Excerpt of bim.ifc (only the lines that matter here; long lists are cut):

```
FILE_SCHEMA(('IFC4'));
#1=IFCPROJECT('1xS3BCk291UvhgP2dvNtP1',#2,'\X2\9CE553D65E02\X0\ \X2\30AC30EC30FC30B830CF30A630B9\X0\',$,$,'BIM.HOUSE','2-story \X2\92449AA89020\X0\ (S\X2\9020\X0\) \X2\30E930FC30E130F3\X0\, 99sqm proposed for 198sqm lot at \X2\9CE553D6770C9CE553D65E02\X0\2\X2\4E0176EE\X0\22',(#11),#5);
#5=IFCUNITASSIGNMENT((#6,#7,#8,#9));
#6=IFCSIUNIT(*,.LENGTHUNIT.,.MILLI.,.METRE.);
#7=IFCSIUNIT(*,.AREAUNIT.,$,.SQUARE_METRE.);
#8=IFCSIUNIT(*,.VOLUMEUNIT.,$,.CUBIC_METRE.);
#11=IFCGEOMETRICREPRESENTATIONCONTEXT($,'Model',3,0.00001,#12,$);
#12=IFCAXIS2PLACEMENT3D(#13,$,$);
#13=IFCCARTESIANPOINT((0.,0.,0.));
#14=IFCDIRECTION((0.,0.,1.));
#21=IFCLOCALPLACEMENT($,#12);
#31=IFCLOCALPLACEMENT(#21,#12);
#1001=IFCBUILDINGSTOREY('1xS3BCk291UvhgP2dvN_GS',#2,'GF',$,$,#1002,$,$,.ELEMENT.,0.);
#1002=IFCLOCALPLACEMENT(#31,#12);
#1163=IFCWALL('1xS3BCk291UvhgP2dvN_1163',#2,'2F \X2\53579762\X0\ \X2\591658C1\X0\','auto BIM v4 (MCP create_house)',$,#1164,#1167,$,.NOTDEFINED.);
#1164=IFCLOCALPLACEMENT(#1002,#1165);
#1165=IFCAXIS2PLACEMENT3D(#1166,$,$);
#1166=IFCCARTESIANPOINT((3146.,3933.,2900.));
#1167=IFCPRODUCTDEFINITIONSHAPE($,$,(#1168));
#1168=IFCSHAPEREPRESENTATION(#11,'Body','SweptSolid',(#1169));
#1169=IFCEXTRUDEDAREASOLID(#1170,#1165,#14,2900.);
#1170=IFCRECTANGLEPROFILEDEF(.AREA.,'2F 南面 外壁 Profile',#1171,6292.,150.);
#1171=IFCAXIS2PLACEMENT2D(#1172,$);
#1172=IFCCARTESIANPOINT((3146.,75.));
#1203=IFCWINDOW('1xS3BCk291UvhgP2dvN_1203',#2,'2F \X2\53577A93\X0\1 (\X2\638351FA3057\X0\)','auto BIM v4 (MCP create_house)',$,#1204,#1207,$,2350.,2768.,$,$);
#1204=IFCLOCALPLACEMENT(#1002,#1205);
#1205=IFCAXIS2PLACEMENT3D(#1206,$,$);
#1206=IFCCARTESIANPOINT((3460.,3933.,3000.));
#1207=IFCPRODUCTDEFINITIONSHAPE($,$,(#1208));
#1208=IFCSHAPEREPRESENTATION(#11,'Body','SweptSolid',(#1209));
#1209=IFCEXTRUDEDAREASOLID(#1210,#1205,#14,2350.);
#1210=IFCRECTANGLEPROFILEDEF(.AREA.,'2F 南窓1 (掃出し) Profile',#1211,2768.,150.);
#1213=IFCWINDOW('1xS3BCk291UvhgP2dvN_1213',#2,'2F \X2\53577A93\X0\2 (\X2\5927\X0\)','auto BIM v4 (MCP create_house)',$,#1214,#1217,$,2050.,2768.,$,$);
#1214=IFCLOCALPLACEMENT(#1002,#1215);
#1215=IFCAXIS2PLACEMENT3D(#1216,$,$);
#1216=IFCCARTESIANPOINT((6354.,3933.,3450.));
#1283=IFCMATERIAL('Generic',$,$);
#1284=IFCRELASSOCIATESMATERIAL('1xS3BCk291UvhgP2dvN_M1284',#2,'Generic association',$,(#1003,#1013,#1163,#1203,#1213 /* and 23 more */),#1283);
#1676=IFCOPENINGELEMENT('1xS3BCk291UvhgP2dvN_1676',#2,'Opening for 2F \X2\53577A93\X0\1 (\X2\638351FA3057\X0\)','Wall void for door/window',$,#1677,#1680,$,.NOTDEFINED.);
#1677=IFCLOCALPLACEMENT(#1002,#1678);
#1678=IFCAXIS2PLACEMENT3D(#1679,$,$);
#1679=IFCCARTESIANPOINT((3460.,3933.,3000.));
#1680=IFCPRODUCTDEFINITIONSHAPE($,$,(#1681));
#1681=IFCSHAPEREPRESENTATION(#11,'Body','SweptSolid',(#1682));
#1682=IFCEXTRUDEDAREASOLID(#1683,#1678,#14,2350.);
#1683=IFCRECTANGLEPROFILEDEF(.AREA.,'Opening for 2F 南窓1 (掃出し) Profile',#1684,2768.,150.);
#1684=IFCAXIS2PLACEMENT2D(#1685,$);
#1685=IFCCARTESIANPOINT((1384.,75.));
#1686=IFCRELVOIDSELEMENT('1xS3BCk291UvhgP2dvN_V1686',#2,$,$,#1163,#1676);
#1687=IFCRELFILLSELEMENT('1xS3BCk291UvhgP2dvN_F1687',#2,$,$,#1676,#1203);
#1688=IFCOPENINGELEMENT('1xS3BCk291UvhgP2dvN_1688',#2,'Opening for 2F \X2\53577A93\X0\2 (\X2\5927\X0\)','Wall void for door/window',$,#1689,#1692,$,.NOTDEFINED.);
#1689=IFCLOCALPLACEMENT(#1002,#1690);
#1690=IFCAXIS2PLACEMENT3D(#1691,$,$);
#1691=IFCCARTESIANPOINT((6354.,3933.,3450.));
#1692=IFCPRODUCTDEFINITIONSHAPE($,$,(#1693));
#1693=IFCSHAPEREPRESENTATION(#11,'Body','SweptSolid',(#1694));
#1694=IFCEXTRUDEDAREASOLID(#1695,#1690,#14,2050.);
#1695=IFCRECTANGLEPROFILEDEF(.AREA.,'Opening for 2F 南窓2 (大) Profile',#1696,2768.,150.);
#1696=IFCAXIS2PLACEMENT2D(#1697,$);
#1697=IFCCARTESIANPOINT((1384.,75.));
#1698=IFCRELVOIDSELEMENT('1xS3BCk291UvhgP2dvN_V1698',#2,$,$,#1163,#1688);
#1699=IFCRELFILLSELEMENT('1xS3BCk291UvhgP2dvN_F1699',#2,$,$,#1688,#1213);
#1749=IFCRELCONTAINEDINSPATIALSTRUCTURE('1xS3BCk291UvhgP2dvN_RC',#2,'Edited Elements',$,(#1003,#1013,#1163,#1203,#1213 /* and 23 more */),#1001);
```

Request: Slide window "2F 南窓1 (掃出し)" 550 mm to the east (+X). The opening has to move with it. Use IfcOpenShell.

```python
import ifcopenshell
import ifcopenshell.api.geometry
import ifcopenshell.util.placement
import ifcopenshell.util.unit

model = ifcopenshell.open("bim.ifc")
unit_scale = ifcopenshell.util.unit.calculate_unit_scale(model)

window = model.by_guid("1xS3BCk291UvhgP2dvN_1203")
opening = window.FillsVoids[0].RelatingOpeningElement
wall = opening.VoidsElements[0].RelatingBuildingElement

wall_matrix = ifcopenshell.util.placement.get_local_placement(wall.ObjectPlacement)
shift = wall_matrix[:3, 0] * 0.55 / unit_scale
before = ifcopenshell.util.placement.get_local_placement(window.ObjectPlacement)[:3, 3].copy()

# The window is not placed relative to its opening, so move both.
for product in (opening, window):
    matrix = ifcopenshell.util.placement.get_local_placement(product.ObjectPlacement)
    matrix[:3, 3] += shift
    ifcopenshell.api.geometry.edit_object_placement(model, product=product, matrix=matrix, is_si=False)

after = ifcopenshell.util.placement.get_local_placement(window.ObjectPlacement)[:3, 3]
print("window moved by", (after - before).round(3) + 0.0)

model.write("bim_updated.ifc")
```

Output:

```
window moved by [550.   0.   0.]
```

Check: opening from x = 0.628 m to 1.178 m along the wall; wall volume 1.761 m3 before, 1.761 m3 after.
